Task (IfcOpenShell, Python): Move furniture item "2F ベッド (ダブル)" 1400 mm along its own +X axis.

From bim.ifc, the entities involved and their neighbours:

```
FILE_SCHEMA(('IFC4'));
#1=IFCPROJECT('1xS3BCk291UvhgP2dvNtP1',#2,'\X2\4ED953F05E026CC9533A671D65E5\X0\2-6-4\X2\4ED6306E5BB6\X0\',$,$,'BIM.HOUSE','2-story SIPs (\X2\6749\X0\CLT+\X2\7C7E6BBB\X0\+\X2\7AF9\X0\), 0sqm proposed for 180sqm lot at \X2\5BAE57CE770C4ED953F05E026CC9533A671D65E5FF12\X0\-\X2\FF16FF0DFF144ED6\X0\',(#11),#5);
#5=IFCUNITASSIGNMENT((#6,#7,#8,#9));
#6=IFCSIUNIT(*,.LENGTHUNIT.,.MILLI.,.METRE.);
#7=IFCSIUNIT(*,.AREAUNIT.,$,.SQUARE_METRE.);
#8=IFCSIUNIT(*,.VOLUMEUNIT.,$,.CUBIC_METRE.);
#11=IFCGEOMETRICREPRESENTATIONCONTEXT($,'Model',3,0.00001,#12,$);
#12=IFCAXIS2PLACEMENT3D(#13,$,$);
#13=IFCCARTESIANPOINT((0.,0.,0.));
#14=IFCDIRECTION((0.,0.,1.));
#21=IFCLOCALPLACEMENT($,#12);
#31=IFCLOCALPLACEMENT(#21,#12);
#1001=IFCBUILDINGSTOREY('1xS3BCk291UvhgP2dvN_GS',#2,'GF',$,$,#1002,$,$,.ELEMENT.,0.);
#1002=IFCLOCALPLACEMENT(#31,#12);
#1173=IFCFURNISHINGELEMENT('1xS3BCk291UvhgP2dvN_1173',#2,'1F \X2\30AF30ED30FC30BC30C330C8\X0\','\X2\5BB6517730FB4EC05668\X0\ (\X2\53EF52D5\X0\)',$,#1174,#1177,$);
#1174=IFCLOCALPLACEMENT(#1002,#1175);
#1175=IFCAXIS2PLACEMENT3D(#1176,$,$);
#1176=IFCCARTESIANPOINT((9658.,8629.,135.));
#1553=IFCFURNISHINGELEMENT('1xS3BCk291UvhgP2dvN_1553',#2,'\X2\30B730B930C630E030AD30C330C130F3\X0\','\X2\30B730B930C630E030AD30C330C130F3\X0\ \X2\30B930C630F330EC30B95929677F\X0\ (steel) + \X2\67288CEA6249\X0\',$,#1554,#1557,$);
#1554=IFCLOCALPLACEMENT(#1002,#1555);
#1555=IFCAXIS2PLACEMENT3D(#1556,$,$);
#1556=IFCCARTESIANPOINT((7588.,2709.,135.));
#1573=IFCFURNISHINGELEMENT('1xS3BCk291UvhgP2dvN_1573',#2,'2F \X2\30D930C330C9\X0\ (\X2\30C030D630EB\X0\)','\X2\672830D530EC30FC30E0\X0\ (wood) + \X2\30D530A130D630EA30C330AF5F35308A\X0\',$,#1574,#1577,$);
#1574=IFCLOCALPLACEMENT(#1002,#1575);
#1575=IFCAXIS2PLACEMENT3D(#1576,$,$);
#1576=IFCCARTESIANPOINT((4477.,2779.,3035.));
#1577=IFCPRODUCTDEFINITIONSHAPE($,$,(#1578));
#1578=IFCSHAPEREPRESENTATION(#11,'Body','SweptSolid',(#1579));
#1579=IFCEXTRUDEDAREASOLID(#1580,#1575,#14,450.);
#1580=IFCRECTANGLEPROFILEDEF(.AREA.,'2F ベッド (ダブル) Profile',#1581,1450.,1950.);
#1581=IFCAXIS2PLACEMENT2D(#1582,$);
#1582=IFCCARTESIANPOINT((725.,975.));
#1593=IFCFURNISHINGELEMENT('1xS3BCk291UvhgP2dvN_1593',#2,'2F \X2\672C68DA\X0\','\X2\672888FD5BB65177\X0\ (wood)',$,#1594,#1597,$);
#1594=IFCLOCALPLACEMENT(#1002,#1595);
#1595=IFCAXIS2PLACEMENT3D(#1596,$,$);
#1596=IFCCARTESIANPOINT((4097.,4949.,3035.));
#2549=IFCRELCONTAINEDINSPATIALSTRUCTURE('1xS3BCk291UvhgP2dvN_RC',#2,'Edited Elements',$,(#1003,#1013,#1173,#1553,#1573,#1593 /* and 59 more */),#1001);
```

```python
import ifcopenshell
import ifcopenshell.api.geometry
import ifcopenshell.util.placement
import ifcopenshell.util.unit

model = ifcopenshell.open("bim.ifc")
unit_scale = ifcopenshell.util.unit.calculate_unit_scale(model)

item = model.by_id(1573)
matrix = ifcopenshell.util.placement.get_local_placement(item.ObjectPlacement)
matrix[:3, 3] += matrix[:3, 0] * 1.4 / unit_scale
ifcopenshell.api.geometry.edit_object_placement(model, product=item, matrix=matrix, is_si=False)

print(ifcopenshell.util.placement.get_local_placement(item.ObjectPlacement).round(3) + 0.0)

model.write("bim_rev.ifc")
```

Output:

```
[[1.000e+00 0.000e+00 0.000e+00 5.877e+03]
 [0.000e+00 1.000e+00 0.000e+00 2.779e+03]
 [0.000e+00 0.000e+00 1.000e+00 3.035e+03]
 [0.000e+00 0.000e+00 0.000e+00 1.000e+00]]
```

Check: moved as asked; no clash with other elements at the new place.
